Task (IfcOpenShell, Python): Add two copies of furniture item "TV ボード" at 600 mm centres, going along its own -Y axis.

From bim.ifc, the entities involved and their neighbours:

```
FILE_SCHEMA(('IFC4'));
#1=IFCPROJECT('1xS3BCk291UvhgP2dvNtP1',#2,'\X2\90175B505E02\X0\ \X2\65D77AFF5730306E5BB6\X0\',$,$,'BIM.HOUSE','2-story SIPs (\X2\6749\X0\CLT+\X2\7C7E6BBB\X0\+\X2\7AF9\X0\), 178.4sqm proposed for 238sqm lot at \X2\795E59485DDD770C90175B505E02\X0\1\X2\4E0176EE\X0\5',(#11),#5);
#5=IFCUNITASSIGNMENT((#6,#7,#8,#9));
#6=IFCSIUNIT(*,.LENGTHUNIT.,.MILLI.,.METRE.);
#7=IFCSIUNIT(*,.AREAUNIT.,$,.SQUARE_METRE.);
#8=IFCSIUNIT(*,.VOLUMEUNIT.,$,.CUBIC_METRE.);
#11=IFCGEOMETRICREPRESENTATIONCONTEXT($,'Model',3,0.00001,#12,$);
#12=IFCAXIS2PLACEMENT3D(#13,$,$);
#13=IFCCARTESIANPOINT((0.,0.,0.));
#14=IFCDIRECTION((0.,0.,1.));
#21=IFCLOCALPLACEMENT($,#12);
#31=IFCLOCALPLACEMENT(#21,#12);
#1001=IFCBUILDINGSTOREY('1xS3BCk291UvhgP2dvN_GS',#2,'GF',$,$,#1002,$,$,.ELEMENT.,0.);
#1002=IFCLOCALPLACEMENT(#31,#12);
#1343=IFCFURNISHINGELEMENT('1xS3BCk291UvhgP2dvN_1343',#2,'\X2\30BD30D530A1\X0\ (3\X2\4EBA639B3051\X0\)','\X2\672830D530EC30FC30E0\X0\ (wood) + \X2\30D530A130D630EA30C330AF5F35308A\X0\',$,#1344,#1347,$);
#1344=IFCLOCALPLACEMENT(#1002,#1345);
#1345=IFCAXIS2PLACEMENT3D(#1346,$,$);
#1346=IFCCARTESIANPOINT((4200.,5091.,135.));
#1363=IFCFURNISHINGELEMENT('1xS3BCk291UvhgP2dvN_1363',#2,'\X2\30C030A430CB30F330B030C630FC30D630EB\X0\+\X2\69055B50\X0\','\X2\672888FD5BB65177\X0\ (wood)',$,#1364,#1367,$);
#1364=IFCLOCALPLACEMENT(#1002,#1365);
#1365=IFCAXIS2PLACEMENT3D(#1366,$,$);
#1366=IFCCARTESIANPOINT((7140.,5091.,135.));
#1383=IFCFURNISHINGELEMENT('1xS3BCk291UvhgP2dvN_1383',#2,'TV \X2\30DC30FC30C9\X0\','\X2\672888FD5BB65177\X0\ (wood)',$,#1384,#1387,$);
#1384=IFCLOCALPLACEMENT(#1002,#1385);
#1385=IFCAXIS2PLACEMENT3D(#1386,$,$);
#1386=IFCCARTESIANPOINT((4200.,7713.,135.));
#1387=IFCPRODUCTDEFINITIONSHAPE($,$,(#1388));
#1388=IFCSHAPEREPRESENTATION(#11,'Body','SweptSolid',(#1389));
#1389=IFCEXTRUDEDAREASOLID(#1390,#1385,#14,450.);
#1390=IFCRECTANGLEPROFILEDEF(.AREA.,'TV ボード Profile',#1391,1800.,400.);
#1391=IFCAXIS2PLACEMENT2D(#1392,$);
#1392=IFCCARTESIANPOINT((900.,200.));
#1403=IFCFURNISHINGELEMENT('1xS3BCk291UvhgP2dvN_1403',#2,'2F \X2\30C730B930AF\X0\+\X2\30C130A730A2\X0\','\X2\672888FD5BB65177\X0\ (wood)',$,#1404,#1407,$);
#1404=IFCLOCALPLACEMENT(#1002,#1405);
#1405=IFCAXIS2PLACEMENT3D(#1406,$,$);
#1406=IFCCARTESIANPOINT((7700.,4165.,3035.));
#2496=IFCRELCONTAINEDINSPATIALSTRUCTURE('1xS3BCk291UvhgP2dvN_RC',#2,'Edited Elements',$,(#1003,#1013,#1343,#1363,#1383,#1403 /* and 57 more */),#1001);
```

```python
import ifcopenshell
import ifcopenshell.api.geometry
import ifcopenshell.api.root
import ifcopenshell.util.element
import ifcopenshell.util.placement
import ifcopenshell.util.unit

model = ifcopenshell.open("bim.ifc")
unit_scale = ifcopenshell.util.unit.calculate_unit_scale(model)


def reuse_history(source, copy):
    """copy_class also copies each property set's owner history, people and application; keep the originals."""
    for rel in copy.IsDefinedBy:
        if rel.is_a("IfcRelDefinesByProperties") and (history := rel.RelatingPropertyDefinition.OwnerHistory):
            rel.RelatingPropertyDefinition.OwnerHistory = source.OwnerHistory
            ifcopenshell.util.element.remove_deep2(model, history)


source = model.by_id(1383)
base = ifcopenshell.util.placement.get_local_placement(source.ObjectPlacement)
step = -base[:3, 1] * 0.6 / unit_scale

for i in range(1, 3):
    copy = ifcopenshell.api.root.copy_class(model, product=source)
    copy.Representation = ifcopenshell.util.element.copy_deep(
        model, source.Representation, exclude=["IfcGeometricRepresentationContext", "IfcRepresentationMap"]
    )
    reuse_history(source, copy)
    matrix = base.copy()
    matrix[:3, 3] += i * step
    print("added at", matrix[:3, 3].round(3) + 0.0)
    ifcopenshell.api.geometry.edit_object_placement(model, product=copy, matrix=matrix, is_si=False)

model.write("bim_rev.ifc")
```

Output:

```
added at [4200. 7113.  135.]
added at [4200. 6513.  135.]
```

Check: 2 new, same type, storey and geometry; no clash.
